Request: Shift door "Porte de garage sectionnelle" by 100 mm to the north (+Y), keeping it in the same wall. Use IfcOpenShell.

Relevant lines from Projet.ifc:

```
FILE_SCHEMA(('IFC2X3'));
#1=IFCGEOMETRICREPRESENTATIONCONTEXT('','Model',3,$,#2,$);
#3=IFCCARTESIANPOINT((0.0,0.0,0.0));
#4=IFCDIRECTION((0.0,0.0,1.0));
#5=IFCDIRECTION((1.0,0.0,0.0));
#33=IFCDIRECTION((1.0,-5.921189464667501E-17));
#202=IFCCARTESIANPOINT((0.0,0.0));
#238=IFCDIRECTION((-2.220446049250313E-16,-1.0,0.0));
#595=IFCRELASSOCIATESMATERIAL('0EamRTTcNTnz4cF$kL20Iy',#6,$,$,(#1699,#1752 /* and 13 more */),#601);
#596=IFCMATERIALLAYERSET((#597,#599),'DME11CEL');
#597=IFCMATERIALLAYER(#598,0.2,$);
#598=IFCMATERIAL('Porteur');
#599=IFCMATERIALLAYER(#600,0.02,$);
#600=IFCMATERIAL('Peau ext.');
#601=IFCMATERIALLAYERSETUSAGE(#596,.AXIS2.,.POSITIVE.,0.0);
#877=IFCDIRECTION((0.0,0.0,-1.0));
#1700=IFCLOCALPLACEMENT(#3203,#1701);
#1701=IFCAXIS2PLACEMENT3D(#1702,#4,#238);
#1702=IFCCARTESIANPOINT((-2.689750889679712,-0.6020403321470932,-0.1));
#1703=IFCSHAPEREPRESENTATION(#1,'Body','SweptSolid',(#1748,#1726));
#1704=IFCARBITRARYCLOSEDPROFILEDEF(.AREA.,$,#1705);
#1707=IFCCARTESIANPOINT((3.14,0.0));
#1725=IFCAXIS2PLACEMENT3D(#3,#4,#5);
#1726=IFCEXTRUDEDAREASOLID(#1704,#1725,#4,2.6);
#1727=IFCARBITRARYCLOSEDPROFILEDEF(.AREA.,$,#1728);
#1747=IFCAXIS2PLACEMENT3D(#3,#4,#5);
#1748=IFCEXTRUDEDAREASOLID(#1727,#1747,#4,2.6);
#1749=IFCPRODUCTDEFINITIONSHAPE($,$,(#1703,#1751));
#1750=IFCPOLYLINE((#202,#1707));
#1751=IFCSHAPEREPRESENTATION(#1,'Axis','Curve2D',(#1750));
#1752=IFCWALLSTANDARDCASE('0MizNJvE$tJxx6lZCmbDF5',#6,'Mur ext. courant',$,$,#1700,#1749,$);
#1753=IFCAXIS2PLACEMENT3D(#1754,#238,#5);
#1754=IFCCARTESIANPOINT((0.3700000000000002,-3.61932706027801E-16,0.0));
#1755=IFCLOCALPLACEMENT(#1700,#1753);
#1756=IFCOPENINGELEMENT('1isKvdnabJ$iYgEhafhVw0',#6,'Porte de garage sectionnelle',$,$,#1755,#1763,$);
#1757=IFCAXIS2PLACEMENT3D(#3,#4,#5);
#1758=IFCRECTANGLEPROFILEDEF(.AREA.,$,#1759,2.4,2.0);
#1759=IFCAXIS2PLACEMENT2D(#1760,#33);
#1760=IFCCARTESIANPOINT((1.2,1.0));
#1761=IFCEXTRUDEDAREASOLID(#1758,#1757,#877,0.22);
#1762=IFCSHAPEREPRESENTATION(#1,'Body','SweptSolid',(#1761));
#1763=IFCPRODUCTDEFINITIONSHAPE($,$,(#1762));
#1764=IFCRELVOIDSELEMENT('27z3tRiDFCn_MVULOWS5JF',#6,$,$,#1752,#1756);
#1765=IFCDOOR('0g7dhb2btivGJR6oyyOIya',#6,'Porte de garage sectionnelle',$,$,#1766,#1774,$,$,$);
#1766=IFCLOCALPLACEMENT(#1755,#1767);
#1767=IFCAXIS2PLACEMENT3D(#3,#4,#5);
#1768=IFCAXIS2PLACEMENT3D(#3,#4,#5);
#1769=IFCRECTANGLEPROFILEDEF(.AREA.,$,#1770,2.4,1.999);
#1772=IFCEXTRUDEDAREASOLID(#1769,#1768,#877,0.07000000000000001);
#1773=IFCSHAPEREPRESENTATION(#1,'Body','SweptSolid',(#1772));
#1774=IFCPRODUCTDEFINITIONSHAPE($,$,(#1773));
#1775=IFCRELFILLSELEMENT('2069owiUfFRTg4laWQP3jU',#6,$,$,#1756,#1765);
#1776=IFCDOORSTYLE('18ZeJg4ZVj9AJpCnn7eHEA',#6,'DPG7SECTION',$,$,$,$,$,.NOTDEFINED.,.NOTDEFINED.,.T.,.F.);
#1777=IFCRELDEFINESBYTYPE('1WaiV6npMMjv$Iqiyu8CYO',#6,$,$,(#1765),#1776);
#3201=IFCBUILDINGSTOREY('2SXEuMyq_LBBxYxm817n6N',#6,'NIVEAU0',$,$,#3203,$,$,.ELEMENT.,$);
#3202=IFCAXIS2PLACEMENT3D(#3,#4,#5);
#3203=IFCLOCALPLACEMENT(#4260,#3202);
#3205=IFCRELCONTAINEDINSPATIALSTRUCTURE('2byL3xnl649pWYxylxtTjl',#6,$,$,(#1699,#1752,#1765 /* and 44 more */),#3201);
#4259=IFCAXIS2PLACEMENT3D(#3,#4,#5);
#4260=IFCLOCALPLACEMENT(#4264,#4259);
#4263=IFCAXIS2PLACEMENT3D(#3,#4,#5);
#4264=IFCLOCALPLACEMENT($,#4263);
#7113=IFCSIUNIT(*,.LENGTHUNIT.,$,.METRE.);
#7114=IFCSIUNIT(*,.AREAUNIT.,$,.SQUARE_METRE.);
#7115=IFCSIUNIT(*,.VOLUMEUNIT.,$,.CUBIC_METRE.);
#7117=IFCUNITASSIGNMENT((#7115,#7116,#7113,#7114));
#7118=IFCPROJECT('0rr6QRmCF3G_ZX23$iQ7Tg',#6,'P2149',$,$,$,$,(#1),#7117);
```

```python
import ifcopenshell
import ifcopenshell.api.geometry
import ifcopenshell.util.placement
import ifcopenshell.util.unit

model = ifcopenshell.open("Projet.ifc")
unit_scale = ifcopenshell.util.unit.calculate_unit_scale(model)

door = model.by_guid("0g7dhb2btivGJR6oyyOIya")
opening = door.FillsVoids[0].RelatingOpeningElement
wall = opening.VoidsElements[0].RelatingBuildingElement

wall_matrix = ifcopenshell.util.placement.get_local_placement(wall.ObjectPlacement)
shift = wall_matrix[:3, 0] * -0.1 / unit_scale
before = ifcopenshell.util.placement.get_local_placement(door.ObjectPlacement)[:3, 3].copy()

# The door is placed relative to its opening, so it follows when the opening moves.
matrix = ifcopenshell.util.placement.get_local_placement(opening.ObjectPlacement)
matrix[:3, 3] += shift
ifcopenshell.api.geometry.edit_object_placement(
    model, product=opening, matrix=matrix, is_si=False, should_transform_children=True
)

after = ifcopenshell.util.placement.get_local_placement(door.ObjectPlacement)[:3, 3]
print("door moved by", (after - before).round(3) + 0.0)

model.write("Projet_v2.ifc")
```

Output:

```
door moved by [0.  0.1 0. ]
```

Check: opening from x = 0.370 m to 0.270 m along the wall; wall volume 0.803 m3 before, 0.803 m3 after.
